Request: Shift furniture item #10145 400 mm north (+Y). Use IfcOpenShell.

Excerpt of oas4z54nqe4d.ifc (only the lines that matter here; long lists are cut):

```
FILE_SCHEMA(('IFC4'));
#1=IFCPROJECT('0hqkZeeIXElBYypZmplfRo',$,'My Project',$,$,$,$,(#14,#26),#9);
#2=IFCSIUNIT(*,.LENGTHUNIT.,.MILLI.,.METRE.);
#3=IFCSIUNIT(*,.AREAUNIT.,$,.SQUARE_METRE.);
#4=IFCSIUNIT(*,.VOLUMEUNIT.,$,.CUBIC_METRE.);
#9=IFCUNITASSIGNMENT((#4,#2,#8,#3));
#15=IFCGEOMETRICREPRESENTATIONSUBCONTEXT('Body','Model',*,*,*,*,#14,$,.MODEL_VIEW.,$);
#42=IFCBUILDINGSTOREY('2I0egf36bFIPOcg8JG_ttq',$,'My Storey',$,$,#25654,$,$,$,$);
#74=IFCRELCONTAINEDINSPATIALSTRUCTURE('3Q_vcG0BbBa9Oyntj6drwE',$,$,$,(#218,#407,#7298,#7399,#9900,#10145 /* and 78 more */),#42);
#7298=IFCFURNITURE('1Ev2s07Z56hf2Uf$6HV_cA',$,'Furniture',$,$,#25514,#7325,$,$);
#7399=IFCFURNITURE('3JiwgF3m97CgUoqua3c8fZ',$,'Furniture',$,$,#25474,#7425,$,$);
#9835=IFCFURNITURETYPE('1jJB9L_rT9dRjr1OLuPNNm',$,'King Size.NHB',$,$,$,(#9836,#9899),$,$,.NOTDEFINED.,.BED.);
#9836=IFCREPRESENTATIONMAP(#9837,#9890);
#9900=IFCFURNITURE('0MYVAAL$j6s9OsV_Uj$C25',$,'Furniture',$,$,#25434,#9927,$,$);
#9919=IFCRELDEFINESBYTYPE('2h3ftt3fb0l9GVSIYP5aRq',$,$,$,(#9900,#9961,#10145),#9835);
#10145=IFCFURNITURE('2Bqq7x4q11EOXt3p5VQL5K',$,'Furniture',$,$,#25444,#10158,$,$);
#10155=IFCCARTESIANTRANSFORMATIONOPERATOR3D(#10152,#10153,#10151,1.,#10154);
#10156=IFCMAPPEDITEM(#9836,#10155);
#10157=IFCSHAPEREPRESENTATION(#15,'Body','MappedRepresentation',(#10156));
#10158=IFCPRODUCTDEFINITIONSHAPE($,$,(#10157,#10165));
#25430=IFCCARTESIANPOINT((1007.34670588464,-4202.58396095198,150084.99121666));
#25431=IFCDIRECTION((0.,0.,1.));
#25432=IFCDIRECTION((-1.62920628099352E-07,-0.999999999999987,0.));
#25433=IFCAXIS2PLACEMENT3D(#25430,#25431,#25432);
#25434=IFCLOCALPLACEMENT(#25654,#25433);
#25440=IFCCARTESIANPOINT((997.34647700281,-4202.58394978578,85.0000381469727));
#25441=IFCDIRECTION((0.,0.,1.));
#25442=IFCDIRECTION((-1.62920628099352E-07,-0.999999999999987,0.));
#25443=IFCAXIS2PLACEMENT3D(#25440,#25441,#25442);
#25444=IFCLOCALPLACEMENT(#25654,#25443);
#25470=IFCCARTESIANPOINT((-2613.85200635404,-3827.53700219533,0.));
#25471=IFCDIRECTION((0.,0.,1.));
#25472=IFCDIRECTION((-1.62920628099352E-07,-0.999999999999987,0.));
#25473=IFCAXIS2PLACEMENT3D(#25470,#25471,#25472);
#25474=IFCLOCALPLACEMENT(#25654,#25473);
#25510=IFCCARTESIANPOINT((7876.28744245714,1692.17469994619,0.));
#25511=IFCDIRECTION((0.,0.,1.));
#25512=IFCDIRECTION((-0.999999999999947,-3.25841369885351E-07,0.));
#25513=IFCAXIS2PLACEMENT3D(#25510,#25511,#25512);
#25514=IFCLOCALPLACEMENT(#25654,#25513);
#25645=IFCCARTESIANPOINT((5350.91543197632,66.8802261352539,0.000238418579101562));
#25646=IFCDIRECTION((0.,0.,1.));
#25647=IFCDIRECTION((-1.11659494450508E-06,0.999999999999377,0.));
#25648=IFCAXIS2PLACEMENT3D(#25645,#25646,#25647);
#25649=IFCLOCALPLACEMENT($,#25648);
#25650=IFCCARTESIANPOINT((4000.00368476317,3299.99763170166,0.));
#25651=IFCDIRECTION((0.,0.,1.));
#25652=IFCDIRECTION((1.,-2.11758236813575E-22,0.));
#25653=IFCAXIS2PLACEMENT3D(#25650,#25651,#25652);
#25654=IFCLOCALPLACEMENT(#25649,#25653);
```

```python
import ifcopenshell
import ifcopenshell.api.geometry
import ifcopenshell.util.placement
import ifcopenshell.util.unit

model = ifcopenshell.open("oas4z54nqe4d.ifc")
unit_scale = ifcopenshell.util.unit.calculate_unit_scale(model)

item = model.by_guid("2Bqq7x4q11EOXt3p5VQL5K")
matrix = ifcopenshell.util.placement.get_local_placement(item.ObjectPlacement)
matrix[1, 3] += 0.4 / unit_scale
ifcopenshell.api.geometry.edit_object_placement(model, product=item, matrix=matrix, is_si=False)

print(ifcopenshell.util.placement.get_local_placement(item.ObjectPlacement).round(3) + 0.0)

model.write("oas4z54nqe4d_edited.ifc")
```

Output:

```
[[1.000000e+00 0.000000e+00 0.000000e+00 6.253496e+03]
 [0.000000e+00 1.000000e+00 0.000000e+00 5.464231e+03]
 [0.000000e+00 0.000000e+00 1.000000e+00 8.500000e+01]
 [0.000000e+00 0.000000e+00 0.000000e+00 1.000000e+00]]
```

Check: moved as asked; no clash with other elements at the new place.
